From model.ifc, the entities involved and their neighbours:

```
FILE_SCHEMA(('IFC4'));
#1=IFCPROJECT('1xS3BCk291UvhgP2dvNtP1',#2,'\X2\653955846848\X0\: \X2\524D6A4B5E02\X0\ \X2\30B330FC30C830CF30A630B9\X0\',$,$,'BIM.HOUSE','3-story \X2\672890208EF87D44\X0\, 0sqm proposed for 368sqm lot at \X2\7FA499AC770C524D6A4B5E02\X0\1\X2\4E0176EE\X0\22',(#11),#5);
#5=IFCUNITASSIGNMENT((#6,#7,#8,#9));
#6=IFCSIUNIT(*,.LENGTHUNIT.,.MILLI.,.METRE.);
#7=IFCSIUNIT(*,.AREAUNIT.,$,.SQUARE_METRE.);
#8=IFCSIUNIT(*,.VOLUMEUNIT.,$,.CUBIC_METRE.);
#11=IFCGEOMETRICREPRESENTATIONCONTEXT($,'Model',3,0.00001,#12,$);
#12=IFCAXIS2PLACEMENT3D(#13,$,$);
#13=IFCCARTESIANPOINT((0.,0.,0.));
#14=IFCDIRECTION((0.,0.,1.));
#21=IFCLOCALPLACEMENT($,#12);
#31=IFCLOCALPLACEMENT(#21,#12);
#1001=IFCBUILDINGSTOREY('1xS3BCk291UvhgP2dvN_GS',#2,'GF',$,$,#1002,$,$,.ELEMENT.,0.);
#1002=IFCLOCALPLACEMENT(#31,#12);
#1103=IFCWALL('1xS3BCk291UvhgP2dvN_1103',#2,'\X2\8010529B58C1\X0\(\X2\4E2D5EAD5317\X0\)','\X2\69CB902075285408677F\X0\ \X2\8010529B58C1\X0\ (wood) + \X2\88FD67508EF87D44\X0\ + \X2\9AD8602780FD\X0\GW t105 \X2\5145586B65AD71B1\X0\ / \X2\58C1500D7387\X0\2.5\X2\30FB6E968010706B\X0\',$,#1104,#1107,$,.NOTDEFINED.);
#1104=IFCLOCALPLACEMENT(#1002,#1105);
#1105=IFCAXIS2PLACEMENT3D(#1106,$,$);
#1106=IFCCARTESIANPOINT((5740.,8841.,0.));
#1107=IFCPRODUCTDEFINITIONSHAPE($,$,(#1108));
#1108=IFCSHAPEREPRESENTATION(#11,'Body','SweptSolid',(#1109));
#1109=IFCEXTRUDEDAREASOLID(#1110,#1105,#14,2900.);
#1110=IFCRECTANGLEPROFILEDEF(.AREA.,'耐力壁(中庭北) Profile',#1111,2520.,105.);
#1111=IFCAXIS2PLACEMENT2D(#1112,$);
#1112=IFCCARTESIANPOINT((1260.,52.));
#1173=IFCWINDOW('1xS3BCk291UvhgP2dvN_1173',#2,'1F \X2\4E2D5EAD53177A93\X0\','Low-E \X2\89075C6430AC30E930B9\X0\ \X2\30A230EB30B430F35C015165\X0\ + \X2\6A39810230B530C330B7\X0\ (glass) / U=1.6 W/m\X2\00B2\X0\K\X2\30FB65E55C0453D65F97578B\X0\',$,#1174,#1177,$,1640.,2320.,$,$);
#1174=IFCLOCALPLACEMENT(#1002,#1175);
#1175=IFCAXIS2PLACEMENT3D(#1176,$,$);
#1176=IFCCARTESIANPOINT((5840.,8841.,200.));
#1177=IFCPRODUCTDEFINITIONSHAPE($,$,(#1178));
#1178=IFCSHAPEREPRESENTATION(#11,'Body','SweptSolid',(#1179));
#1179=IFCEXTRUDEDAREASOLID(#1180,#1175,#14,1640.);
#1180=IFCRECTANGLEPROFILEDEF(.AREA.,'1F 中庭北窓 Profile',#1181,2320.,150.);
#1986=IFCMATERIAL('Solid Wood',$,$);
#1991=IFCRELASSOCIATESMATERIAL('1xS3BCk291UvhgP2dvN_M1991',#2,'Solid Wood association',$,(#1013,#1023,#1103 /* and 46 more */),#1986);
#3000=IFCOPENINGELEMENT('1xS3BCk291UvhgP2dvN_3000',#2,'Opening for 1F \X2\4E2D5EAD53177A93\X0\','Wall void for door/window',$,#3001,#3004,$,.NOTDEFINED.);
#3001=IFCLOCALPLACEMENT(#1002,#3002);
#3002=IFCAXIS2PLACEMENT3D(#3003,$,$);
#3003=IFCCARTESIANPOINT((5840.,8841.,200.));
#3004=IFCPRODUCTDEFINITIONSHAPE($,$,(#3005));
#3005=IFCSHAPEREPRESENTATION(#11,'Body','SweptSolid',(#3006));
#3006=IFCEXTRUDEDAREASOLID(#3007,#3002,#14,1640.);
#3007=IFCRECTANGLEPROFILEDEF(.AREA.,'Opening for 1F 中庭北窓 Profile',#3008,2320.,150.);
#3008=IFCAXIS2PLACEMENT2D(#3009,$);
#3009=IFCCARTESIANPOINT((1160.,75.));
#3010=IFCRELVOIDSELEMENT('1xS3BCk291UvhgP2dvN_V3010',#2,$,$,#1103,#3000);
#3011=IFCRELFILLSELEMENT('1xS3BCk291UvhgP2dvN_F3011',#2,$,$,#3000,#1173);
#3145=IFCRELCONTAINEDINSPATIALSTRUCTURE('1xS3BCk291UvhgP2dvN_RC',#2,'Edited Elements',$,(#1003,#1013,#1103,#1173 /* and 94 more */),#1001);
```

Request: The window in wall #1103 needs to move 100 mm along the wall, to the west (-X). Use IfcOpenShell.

```python
import ifcopenshell
import ifcopenshell.api.geometry
import ifcopenshell.util.placement

model = ifcopenshell.open("model.ifc")

window = model.by_guid("1xS3BCk291UvhgP2dvN_1173")
opening = window.FillsVoids[0].RelatingOpeningElement
wall = opening.VoidsElements[0].RelatingBuildingElement

wall_matrix = ifcopenshell.util.placement.get_local_placement(wall.ObjectPlacement)
shift = wall_matrix[:3, 0] * -100.0
before = ifcopenshell.util.placement.get_local_placement(window.ObjectPlacement)[:3, 3].copy()

# The window is not placed relative to its opening, so move both.
for product in (opening, window):
    matrix = ifcopenshell.util.placement.get_local_placement(product.ObjectPlacement)
    matrix[:3, 3] += shift
    ifcopenshell.api.geometry.edit_object_placement(model, product=product, matrix=matrix, is_si=False)

after = ifcopenshell.util.placement.get_local_placement(window.ObjectPlacement)[:3, 3]
print("window moved by", (after - before).round(3) + 0.0)

model.write("model_updated.ifc")
```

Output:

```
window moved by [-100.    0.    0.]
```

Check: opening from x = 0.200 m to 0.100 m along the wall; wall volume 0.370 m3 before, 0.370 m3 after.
